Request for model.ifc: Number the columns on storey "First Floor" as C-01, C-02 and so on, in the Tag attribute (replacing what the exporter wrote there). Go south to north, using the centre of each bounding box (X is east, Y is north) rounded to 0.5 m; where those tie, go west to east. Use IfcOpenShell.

First a look at what the model holds.

```python
import ifcopenshell
import ifcopenshell.util.element
import ifcopenshell.util.placement

model = ifcopenshell.open("model.ifc")
print(model.schema)
storey = next(s for s in model.by_type("IfcBuildingStorey") if s.Name == "First Floor")
columns = [e for e in ifcopenshell.util.element.get_decomposition(storey) if e.is_a("IfcColumn")]
for e in sorted(columns, key=lambda e: e.id()):
    origin = ifcopenshell.util.placement.get_local_placement(e.ObjectPlacement)[:3, 3]
    print(e.id(), e.Tag, e.Name, origin.round(2) + 0.0, sep=" | ")
```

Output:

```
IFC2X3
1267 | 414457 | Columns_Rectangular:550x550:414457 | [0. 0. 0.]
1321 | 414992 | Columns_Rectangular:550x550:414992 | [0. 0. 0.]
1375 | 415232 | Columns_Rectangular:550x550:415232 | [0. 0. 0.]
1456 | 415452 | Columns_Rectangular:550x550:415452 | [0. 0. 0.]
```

```python
import ifcopenshell
import ifcopenshell.geom
import ifcopenshell.util.element
import ifcopenshell.util.shape

model = ifcopenshell.open("model.ifc")
settings = ifcopenshell.geom.settings()
settings.set("use-world-coords", True)


def centre(element):
    shape = ifcopenshell.geom.create_shape(settings, element)
    return ifcopenshell.util.shape.get_bbox_centroid(shape.geometry)


storey = next(s for s in model.by_type("IfcBuildingStorey") if s.Name == "First Floor")
columns = [e for e in ifcopenshell.util.element.get_decomposition(storey) if e.is_a("IfcColumn")]

# Insertion points can sit at a corner or the storey origin, so sort by the geometry (in metres).
centres = {e: centre(e) for e in columns}
columns.sort(key=lambda e: (round(centres[e][1] / 0.5), centres[e][0]))

for i, e in enumerate(columns, start=1):
    number = f"C-{i:02d}"
    e.Tag = number
    print(e.id(), number)

model.write("model-out.ifc")
```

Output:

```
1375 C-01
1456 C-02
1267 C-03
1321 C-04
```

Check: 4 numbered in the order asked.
